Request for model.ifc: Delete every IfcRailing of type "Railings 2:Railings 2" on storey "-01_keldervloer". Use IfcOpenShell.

First a look at what the model holds.

```python
import ifcopenshell
import ifcopenshell.util.element

model = ifcopenshell.open("model.ifc")
print(model.schema)
storey = next(s for s in model.by_type("IfcBuildingStorey") if s.Name == "-01_keldervloer")
railings = [e for e in ifcopenshell.util.element.get_decomposition(storey) if e.is_a("IfcRailing")]
seen = {}
for e in railings:
    element_type = ifcopenshell.util.element.get_type(e)
    name = element_type.Name if element_type not in (None, e) else None
    seen[name] = seen.get(name, 0) + 1
for name, count in sorted(seen.items(), key=str):
    print(count, "x", name)
```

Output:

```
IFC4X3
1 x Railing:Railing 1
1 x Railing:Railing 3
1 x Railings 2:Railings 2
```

```python
import ifcopenshell
import ifcopenshell.api.root
import ifcopenshell.util.element

model = ifcopenshell.open("model.ifc")

storey = next(s for s in model.by_type("IfcBuildingStorey") if s.Name == "-01_keldervloer")
railings = [e for e in ifcopenshell.util.element.get_decomposition(storey) if e.is_a("IfcRailing")]
targets = [e for e in railings if (t := ifcopenshell.util.element.get_type(e)) not in (None, e) and t.Name == "Railings 2:Railings 2"]

for e in targets:
    ifcopenshell.api.root.remove_product(model, product=e)
print(len(targets), "removed")

model.write("model-out.ifc")
```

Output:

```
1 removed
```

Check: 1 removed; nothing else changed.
